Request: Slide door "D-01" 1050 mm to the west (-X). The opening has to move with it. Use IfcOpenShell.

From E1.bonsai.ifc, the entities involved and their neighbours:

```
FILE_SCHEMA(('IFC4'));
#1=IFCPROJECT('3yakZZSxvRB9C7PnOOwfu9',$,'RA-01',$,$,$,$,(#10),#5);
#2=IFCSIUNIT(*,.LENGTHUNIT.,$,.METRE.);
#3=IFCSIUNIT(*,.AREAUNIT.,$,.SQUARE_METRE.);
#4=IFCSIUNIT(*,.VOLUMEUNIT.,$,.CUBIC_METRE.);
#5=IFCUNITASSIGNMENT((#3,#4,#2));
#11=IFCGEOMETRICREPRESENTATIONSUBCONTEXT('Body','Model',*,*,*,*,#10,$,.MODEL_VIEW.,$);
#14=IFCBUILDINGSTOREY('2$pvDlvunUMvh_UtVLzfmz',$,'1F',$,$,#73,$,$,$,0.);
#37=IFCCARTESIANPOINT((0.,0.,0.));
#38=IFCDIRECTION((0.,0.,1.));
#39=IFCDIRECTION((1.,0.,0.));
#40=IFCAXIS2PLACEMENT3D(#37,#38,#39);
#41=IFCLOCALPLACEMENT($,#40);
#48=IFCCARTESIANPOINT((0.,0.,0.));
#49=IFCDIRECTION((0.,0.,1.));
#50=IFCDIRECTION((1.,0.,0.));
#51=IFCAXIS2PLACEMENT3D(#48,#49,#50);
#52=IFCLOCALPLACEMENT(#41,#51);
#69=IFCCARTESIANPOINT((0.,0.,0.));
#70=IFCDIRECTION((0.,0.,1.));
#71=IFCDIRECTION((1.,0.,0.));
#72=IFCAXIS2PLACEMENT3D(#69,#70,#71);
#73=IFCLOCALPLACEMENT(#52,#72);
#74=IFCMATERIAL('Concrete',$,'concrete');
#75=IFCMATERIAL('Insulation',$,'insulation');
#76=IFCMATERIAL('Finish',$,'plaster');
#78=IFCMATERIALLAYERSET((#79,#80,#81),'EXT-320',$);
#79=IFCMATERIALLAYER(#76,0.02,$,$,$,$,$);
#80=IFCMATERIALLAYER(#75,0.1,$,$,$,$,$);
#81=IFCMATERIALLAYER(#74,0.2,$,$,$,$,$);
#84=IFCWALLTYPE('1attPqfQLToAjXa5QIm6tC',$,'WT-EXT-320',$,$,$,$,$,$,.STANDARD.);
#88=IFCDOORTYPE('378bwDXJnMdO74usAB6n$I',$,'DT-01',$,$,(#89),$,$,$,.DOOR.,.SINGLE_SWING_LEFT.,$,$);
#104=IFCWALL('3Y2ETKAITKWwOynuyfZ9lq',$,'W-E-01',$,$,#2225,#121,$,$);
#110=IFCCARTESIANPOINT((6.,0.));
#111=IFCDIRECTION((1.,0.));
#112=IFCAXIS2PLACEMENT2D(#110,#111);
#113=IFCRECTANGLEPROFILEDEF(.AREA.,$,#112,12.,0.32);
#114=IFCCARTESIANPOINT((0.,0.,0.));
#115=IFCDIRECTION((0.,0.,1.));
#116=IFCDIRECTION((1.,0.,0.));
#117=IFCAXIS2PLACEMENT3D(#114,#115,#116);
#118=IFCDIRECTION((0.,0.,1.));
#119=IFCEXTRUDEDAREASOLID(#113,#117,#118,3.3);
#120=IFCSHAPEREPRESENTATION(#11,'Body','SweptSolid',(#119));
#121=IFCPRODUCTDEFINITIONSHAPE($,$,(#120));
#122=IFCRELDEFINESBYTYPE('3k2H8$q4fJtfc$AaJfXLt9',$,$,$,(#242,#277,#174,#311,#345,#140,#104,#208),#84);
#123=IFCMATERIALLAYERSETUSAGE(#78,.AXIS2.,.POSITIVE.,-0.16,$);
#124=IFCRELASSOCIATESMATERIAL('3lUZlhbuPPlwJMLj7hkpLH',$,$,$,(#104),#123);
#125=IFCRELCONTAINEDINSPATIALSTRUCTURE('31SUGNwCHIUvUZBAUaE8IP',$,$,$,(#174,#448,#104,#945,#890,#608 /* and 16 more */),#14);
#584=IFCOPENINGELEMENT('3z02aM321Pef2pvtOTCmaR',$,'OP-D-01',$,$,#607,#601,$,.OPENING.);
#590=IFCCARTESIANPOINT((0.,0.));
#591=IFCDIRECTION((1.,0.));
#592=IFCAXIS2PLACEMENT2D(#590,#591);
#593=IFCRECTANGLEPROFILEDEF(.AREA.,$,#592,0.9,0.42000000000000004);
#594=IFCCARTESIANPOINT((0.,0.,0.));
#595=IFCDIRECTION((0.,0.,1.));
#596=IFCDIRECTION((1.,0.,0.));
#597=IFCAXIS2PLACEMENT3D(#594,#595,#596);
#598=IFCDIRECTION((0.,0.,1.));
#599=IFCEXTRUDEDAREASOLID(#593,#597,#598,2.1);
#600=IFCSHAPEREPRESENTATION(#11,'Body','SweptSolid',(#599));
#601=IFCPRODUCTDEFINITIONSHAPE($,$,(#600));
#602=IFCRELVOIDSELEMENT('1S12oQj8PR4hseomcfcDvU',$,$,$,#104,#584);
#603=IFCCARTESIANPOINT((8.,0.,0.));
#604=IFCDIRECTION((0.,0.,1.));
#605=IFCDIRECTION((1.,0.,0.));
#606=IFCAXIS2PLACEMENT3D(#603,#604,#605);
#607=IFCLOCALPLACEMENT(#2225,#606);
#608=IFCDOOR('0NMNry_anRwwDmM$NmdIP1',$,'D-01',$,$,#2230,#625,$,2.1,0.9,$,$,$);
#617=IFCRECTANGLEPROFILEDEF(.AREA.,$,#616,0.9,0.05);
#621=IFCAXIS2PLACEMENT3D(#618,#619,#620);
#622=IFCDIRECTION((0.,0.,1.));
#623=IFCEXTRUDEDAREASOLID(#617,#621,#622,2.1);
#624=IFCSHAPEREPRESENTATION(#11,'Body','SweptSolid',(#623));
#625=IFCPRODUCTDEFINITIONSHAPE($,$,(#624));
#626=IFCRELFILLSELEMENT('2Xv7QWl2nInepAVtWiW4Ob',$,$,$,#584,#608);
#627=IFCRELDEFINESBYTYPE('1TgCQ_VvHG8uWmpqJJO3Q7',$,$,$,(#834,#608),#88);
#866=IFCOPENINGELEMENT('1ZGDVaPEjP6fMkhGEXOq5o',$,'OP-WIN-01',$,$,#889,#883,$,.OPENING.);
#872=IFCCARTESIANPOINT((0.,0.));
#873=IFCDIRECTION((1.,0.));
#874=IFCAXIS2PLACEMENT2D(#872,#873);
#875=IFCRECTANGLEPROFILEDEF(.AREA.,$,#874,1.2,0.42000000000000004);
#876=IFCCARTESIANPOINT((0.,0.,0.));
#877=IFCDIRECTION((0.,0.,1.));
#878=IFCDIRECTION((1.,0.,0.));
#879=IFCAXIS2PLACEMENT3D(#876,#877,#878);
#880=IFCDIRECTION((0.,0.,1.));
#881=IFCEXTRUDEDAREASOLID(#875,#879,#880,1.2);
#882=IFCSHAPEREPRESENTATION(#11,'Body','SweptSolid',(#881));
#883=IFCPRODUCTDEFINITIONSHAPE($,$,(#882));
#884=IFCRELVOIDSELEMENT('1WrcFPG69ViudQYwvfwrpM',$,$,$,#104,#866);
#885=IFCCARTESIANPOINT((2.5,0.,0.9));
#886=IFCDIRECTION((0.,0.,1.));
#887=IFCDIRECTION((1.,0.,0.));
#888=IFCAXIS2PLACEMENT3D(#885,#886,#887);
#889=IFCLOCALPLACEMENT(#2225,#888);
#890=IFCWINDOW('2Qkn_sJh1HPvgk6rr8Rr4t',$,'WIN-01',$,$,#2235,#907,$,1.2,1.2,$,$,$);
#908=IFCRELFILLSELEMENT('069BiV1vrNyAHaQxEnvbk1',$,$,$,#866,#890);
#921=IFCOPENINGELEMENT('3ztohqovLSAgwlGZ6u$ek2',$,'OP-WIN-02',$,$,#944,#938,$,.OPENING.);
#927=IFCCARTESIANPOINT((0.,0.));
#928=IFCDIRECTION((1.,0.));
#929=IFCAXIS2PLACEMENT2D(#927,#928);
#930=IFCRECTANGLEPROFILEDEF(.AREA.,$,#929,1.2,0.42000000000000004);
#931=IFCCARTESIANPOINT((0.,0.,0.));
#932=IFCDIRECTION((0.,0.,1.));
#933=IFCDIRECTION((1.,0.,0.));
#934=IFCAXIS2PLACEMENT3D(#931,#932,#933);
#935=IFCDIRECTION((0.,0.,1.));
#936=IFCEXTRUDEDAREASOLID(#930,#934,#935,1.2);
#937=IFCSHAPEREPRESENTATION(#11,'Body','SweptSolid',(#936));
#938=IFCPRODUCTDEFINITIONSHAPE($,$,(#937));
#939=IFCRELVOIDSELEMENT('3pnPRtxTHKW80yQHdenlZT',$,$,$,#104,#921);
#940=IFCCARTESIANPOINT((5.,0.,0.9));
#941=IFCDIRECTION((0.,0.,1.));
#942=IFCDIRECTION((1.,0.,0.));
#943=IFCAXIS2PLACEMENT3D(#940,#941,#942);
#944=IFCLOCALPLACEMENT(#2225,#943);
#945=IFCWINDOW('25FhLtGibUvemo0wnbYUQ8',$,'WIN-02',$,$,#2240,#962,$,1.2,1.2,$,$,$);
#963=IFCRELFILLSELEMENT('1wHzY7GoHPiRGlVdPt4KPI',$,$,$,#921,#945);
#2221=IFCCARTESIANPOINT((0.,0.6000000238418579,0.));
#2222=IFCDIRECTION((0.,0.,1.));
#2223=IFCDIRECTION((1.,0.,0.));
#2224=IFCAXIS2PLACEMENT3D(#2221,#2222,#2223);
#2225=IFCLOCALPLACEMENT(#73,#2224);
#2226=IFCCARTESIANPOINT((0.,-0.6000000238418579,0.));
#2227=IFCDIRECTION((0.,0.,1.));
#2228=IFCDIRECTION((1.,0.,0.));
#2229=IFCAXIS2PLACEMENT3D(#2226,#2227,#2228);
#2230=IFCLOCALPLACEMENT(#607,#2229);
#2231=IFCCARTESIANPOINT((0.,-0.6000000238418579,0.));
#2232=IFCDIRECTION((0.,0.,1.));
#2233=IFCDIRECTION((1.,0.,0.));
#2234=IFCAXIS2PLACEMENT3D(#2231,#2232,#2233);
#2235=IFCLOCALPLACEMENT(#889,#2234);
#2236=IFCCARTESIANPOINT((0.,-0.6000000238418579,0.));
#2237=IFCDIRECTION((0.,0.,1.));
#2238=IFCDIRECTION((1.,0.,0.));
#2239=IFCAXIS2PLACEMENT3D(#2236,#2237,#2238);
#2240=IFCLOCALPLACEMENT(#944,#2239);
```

```python
import ifcopenshell
import ifcopenshell.api.geometry
import ifcopenshell.util.placement
import ifcopenshell.util.unit

model = ifcopenshell.open("E1.bonsai.ifc")
unit_scale = ifcopenshell.util.unit.calculate_unit_scale(model)

door = model.by_guid("0NMNry_anRwwDmM$NmdIP1")
opening = door.FillsVoids[0].RelatingOpeningElement
wall = opening.VoidsElements[0].RelatingBuildingElement

wall_matrix = ifcopenshell.util.placement.get_local_placement(wall.ObjectPlacement)
shift = wall_matrix[:3, 0] * -1.05 / unit_scale
before = ifcopenshell.util.placement.get_local_placement(door.ObjectPlacement)[:3, 3].copy()

# The door is placed relative to its opening, so it follows when the opening moves.
matrix = ifcopenshell.util.placement.get_local_placement(opening.ObjectPlacement)
matrix[:3, 3] += shift
ifcopenshell.api.geometry.edit_object_placement(
    model, product=opening, matrix=matrix, is_si=False, should_transform_children=True
)

after = ifcopenshell.util.placement.get_local_placement(door.ObjectPlacement)[:3, 3]
print("door moved by", (after - before).round(3) + 0.0)

model.write("E1.bonsai_updated.ifc")
```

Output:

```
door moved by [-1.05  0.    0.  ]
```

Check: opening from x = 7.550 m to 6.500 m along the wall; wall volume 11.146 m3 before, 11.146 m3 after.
